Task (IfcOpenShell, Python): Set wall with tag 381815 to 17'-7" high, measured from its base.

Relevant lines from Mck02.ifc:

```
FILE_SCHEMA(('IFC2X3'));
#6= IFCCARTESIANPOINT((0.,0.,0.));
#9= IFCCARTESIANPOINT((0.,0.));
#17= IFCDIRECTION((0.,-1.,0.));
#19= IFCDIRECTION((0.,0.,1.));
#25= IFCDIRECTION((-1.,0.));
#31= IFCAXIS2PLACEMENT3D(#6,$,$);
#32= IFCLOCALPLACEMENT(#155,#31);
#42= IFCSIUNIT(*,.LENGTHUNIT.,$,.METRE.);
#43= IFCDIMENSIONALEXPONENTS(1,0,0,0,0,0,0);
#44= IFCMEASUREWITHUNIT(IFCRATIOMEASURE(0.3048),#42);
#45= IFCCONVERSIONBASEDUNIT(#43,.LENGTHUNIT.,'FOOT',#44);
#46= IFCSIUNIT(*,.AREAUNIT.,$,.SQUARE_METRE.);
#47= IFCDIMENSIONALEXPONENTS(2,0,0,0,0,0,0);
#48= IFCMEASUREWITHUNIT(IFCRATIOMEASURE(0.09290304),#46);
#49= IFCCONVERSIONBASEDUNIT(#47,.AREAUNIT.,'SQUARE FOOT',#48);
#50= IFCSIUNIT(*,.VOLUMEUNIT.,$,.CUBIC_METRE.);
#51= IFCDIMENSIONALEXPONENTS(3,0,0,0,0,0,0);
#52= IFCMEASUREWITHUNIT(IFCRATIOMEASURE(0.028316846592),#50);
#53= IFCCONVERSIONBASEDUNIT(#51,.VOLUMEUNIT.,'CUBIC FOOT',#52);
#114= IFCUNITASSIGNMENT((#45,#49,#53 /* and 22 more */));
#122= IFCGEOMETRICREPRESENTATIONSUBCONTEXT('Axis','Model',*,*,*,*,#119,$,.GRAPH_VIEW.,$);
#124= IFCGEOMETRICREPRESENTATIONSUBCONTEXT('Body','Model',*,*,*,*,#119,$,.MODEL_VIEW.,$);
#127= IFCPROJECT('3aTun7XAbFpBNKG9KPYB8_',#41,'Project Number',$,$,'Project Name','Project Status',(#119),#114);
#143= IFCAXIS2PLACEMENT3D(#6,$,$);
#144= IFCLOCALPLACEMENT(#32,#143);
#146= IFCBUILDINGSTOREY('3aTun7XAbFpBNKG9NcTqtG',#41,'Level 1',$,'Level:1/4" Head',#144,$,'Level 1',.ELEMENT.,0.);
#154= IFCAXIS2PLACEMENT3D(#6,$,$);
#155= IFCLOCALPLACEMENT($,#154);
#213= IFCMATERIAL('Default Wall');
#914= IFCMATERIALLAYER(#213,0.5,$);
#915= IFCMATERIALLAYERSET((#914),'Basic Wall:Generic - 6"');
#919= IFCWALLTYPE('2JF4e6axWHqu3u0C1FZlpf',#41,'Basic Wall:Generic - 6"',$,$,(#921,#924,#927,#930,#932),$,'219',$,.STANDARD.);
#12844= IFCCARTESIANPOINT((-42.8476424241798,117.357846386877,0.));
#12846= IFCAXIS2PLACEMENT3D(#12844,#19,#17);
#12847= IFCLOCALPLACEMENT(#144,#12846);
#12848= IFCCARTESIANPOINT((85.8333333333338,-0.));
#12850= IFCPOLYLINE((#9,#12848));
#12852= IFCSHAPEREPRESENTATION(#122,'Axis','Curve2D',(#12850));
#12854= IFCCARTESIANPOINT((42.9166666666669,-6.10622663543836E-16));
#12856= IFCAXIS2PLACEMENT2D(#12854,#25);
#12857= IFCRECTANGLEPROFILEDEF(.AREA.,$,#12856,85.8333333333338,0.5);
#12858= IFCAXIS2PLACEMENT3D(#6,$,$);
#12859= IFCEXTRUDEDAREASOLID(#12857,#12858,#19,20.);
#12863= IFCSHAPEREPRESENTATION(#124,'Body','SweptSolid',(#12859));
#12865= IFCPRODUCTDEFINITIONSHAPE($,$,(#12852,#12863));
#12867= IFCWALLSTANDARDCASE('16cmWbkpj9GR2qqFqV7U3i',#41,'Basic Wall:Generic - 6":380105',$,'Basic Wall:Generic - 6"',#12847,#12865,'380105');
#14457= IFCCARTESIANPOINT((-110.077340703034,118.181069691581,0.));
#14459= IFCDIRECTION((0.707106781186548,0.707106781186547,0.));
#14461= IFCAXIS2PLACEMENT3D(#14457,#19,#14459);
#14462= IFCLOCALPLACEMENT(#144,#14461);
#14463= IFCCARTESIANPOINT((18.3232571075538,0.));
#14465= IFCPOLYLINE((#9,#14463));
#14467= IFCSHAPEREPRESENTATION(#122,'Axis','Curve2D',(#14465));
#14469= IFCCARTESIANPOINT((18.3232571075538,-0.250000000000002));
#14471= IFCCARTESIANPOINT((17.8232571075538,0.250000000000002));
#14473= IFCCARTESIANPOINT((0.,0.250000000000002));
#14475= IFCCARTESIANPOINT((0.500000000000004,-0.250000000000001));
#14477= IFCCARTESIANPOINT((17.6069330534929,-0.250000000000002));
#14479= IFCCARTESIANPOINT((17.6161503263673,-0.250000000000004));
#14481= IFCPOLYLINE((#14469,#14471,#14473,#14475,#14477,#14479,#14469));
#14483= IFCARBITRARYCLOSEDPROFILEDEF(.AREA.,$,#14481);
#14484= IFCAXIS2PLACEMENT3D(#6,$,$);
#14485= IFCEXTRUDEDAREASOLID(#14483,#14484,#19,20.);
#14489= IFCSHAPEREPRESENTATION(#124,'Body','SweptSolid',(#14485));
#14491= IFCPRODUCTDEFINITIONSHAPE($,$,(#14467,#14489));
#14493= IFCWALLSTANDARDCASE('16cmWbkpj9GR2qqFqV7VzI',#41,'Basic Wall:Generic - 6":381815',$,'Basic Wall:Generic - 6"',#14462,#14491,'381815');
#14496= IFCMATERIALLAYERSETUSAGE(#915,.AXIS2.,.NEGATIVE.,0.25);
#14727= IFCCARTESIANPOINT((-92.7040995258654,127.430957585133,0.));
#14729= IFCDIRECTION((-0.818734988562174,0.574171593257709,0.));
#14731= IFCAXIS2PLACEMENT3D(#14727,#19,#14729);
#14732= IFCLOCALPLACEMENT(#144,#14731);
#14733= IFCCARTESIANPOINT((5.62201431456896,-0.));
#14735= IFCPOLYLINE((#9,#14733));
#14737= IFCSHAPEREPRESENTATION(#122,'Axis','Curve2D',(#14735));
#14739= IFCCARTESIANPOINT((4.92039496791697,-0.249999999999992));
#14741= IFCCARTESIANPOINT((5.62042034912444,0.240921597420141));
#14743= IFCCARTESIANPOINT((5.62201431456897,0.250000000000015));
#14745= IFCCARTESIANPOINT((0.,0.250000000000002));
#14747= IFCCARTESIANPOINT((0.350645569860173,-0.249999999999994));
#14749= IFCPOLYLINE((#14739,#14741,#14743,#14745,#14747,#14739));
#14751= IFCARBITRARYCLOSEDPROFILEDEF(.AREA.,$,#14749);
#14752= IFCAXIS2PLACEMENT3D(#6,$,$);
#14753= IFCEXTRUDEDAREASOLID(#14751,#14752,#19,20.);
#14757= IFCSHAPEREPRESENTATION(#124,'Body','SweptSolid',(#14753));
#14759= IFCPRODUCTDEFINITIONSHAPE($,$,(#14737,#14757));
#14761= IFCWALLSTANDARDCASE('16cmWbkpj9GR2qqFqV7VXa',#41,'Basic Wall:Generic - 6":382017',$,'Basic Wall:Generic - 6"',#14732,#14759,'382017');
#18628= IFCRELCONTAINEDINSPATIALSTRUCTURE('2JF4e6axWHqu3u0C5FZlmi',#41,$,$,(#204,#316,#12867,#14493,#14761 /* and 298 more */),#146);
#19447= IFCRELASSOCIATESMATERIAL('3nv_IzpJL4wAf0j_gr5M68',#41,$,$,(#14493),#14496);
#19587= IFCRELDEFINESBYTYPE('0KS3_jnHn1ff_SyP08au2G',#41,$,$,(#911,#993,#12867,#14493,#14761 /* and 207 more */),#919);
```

```python
import ifcopenshell
import ifcopenshell.geom
import ifcopenshell.util.representation
import ifcopenshell.util.shape
import ifcopenshell.util.unit

model = ifcopenshell.open("Mck02.ifc")
unit_scale = ifcopenshell.util.unit.calculate_unit_scale(model)
settings = ifcopenshell.geom.settings()


def volume(element):
    """Net volume in cubic metres, openings subtracted."""
    shape = ifcopenshell.geom.create_shape(settings, element)
    return ifcopenshell.util.shape.get_volume(shape.geometry)


wall = model.by_guid("16cmWbkpj9GR2qqFqV7VzI")
before = volume(wall)

body = ifcopenshell.util.representation.get_representation(wall, "Model", "Body")
solid = body.Items[0]
old_height = solid.Depth
solid.Depth = 211 * 0.0254 / unit_scale
after = volume(wall)

print(f"height {old_height:g} -> {solid.Depth:g}, volume {before:.3f} -> {after:.3f} m3")

model.write("Mck02-out.ifc")
```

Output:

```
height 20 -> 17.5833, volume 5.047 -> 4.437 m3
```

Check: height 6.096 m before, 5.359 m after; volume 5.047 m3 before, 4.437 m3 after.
